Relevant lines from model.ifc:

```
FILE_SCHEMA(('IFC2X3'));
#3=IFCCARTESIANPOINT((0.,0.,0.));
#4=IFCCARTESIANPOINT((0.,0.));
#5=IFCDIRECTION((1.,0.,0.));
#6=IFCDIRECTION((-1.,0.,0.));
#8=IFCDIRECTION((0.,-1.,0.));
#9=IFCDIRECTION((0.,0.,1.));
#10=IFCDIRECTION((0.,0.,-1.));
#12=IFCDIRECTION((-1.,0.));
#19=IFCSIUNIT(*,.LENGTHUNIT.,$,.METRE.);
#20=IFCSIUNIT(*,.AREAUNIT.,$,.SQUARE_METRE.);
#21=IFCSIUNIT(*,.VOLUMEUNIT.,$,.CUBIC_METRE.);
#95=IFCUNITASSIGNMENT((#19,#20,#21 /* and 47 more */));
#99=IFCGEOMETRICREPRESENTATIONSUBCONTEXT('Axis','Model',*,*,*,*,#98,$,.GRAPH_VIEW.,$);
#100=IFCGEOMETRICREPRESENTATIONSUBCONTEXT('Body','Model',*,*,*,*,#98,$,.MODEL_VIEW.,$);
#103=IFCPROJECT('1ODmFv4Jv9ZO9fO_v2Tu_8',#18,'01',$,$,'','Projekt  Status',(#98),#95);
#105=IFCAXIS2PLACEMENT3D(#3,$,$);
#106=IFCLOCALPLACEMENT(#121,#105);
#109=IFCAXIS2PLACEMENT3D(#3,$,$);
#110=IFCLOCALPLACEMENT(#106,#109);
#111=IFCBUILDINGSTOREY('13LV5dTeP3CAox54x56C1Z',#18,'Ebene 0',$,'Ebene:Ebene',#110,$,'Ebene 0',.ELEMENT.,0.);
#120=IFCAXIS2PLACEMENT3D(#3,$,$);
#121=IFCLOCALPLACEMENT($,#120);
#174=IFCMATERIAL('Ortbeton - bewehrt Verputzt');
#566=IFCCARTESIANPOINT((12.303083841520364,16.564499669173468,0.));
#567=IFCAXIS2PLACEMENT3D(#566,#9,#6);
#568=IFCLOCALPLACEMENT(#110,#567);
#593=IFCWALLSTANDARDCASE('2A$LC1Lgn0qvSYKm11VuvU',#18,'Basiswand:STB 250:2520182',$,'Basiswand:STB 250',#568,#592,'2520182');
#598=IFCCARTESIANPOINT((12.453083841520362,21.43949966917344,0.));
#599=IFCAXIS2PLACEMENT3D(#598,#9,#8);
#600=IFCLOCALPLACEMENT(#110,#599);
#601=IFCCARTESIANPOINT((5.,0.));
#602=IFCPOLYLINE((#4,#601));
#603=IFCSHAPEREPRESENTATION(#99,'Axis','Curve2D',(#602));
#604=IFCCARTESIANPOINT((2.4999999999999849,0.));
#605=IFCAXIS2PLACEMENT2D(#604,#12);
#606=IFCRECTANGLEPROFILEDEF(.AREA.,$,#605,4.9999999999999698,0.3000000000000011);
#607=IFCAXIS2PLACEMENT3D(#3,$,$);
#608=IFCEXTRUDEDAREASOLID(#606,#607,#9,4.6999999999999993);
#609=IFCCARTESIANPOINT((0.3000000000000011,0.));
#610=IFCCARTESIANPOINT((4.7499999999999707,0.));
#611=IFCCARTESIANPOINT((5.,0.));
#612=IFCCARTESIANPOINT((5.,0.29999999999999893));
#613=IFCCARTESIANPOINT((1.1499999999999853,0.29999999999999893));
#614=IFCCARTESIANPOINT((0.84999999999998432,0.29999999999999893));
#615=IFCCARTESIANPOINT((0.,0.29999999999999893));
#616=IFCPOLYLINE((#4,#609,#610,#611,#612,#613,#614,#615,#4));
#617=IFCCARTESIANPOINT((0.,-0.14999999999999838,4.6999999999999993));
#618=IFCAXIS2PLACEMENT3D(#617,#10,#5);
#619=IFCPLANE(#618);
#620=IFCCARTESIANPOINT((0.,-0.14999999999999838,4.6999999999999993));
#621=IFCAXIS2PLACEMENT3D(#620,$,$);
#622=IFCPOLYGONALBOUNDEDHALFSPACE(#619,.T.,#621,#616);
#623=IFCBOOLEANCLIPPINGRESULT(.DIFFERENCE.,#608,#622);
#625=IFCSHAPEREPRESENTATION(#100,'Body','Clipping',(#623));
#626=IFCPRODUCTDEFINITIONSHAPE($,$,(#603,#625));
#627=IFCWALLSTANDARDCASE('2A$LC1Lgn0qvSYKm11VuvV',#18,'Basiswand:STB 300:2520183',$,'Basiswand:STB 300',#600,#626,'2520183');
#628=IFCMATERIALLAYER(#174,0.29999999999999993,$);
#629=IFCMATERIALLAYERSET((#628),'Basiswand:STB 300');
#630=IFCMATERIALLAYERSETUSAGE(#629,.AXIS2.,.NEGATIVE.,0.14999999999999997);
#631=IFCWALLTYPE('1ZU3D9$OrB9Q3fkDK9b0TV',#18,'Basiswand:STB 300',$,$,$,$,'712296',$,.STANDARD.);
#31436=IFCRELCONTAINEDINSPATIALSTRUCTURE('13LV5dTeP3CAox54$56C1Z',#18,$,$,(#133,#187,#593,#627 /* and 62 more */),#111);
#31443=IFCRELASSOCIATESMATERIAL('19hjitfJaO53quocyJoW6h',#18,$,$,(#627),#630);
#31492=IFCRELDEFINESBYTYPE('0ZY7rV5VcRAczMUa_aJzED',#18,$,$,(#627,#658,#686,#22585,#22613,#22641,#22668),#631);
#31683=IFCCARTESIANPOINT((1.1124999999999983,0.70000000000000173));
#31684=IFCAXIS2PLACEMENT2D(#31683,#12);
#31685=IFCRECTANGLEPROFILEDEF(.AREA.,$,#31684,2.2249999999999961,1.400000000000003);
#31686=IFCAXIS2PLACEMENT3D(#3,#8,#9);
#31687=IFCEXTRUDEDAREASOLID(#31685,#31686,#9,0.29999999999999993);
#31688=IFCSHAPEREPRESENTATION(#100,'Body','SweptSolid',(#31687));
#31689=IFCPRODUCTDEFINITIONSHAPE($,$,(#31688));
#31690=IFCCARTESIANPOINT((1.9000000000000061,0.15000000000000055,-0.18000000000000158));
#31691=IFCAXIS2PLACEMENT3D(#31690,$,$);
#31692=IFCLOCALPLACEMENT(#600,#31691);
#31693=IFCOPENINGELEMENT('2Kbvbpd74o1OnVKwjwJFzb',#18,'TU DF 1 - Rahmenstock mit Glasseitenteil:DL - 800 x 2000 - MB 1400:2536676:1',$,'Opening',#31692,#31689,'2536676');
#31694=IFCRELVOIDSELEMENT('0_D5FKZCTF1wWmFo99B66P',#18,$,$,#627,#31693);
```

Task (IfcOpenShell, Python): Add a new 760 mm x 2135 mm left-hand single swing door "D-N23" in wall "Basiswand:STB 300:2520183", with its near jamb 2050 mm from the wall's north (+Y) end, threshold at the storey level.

```python
import numpy as np
import ifcopenshell
import ifcopenshell.api.feature
import ifcopenshell.api.geometry
import ifcopenshell.api.root
import ifcopenshell.api.spatial
import ifcopenshell.api.type
import ifcopenshell.geom
import ifcopenshell.util.element
import ifcopenshell.util.placement
import ifcopenshell.util.representation
import ifcopenshell.util.shape
import ifcopenshell.util.unit

model = ifcopenshell.open("model.ifc")
unit_scale = ifcopenshell.util.unit.calculate_unit_scale(model)
settings = ifcopenshell.geom.settings()


def volume(element):
    """Net volume in cubic metres, openings subtracted."""
    shape = ifcopenshell.geom.create_shape(settings, element)
    return ifcopenshell.util.shape.get_volume(shape.geometry)


wall = model.by_id(627)
storey = ifcopenshell.util.element.get_container(wall, ifc_class="IfcBuildingStorey")
context = ifcopenshell.util.representation.get_context(model, "Model", "Body", "MODEL_VIEW")
before = volume(wall)

width, height, from_end, sill = 0.76, 2.135, 2.05, 0.0  # metres

# The wall runs along its own X axis, and the end named is its -X end.
wall_shape = ifcopenshell.geom.create_shape(settings, wall)
x, y, z = ifcopenshell.util.shape.get_vertices(wall_shape.geometry).T
start = x.min() + from_end
face, thickness = float(y.min()), float(y.max() - y.min())
wall_matrix = ifcopenshell.util.placement.get_local_placement(wall.ObjectPlacement)
level = ifcopenshell.util.placement.get_local_placement(storey.ObjectPlacement)[2, 3]


def in_wall(x, y):
    """Placement at x, y metres in the wall's axes, at sill height."""
    matrix = wall_matrix.copy()
    matrix[:, 3] = wall_matrix @ np.array([x / unit_scale, y / unit_scale, 0.0, 1.0])
    matrix[2, 3] = level + sill / unit_scale
    return matrix


# Opening: a box that overshoots both wall faces by 50 mm.
opening = ifcopenshell.api.root.create_entity(model, ifc_class="IfcOpeningElement")
box = ifcopenshell.api.geometry.add_wall_representation(
    model, context=context, length=width, height=height, thickness=thickness + 0.1
)
ifcopenshell.api.geometry.assign_representation(model, product=opening, representation=box)
ifcopenshell.api.geometry.edit_object_placement(model, product=opening, matrix=in_wall(start, face - 0.05), is_si=False)
ifcopenshell.api.feature.add_feature(model, feature=opening, element=wall)

door = ifcopenshell.api.root.create_entity(model, ifc_class="IfcDoor", name="D-N23")
door.OverallWidth, door.OverallHeight = width / unit_scale, height / unit_scale
body = ifcopenshell.api.geometry.add_door_representation(
    model,
    context=context,
    overall_width=door.OverallWidth,
    overall_height=door.OverallHeight,
    operation_type="SINGLE_SWING_LEFT",
    lining_properties={"LiningDepth": thickness / unit_scale, "ThresholdDepth": thickness / unit_scale},
)
ifcopenshell.api.geometry.assign_representation(model, product=door, representation=body)
ifcopenshell.api.spatial.assign_container(model, products=[door], relating_structure=storey)
fills = ifcopenshell.api.feature.add_filling(model, opening=opening, element=door)
fills.OwnerHistory = door.OwnerHistory  # required in IFC2X3

# IFC2X3 keeps the operation on the door style.
style = ifcopenshell.api.root.create_entity(model, ifc_class="IfcDoorStyle", name="D-N23")
style.OperationType, style.ConstructionType = "SINGLE_SWING_LEFT", "NOTDEFINED"
style.ParameterTakesPrecedence = style.Sizeable = False
ifcopenshell.api.type.assign_type(model, related_objects=[door], relating_type=style)

# The lining spans the wall, so the door starts at the wall face.
ifcopenshell.api.geometry.edit_object_placement(model, product=door, matrix=in_wall(start, face), is_si=False)

after = volume(wall)

print(f"wall volume {before:.3f} -> {after:.3f} m3")

model.write("model_v2.ifc")
```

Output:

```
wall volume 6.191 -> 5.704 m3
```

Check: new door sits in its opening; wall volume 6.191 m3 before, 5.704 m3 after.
